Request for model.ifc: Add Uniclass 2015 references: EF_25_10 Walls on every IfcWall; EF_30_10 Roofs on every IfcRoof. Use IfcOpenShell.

First a look at what the model holds.

```python
import ifcopenshell

model = ifcopenshell.open("model.ifc")
print(model.schema)
print("classifications:", [c.Name for c in model.by_type("IfcClassification")])
for ifc_class in ("IfcDoor", "IfcRoof", "IfcStair", "IfcWall", "IfcWindow"):
    print(ifc_class, len(model.by_type(ifc_class)))
```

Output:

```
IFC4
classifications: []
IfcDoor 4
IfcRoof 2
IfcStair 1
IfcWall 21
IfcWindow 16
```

```python
import ifcopenshell
import ifcopenshell.api.classification

model = ifcopenshell.open("model.ifc")

system = ifcopenshell.api.classification.add_classification(model, classification="Uniclass 2015")

codes = {
    "IfcWall": ("EF_25_10", "Walls"),
    "IfcRoof": ("EF_30_10", "Roofs"),
}
for ifc_class, (code, name) in codes.items():
    products = model.by_type(ifc_class)
    ifcopenshell.api.classification.add_reference(
        model, products=products, classification=system, identification=code, name=name
    )
    print(code, len(products))

model.write("model-out.ifc")
```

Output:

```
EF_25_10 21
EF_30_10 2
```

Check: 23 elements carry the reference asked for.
